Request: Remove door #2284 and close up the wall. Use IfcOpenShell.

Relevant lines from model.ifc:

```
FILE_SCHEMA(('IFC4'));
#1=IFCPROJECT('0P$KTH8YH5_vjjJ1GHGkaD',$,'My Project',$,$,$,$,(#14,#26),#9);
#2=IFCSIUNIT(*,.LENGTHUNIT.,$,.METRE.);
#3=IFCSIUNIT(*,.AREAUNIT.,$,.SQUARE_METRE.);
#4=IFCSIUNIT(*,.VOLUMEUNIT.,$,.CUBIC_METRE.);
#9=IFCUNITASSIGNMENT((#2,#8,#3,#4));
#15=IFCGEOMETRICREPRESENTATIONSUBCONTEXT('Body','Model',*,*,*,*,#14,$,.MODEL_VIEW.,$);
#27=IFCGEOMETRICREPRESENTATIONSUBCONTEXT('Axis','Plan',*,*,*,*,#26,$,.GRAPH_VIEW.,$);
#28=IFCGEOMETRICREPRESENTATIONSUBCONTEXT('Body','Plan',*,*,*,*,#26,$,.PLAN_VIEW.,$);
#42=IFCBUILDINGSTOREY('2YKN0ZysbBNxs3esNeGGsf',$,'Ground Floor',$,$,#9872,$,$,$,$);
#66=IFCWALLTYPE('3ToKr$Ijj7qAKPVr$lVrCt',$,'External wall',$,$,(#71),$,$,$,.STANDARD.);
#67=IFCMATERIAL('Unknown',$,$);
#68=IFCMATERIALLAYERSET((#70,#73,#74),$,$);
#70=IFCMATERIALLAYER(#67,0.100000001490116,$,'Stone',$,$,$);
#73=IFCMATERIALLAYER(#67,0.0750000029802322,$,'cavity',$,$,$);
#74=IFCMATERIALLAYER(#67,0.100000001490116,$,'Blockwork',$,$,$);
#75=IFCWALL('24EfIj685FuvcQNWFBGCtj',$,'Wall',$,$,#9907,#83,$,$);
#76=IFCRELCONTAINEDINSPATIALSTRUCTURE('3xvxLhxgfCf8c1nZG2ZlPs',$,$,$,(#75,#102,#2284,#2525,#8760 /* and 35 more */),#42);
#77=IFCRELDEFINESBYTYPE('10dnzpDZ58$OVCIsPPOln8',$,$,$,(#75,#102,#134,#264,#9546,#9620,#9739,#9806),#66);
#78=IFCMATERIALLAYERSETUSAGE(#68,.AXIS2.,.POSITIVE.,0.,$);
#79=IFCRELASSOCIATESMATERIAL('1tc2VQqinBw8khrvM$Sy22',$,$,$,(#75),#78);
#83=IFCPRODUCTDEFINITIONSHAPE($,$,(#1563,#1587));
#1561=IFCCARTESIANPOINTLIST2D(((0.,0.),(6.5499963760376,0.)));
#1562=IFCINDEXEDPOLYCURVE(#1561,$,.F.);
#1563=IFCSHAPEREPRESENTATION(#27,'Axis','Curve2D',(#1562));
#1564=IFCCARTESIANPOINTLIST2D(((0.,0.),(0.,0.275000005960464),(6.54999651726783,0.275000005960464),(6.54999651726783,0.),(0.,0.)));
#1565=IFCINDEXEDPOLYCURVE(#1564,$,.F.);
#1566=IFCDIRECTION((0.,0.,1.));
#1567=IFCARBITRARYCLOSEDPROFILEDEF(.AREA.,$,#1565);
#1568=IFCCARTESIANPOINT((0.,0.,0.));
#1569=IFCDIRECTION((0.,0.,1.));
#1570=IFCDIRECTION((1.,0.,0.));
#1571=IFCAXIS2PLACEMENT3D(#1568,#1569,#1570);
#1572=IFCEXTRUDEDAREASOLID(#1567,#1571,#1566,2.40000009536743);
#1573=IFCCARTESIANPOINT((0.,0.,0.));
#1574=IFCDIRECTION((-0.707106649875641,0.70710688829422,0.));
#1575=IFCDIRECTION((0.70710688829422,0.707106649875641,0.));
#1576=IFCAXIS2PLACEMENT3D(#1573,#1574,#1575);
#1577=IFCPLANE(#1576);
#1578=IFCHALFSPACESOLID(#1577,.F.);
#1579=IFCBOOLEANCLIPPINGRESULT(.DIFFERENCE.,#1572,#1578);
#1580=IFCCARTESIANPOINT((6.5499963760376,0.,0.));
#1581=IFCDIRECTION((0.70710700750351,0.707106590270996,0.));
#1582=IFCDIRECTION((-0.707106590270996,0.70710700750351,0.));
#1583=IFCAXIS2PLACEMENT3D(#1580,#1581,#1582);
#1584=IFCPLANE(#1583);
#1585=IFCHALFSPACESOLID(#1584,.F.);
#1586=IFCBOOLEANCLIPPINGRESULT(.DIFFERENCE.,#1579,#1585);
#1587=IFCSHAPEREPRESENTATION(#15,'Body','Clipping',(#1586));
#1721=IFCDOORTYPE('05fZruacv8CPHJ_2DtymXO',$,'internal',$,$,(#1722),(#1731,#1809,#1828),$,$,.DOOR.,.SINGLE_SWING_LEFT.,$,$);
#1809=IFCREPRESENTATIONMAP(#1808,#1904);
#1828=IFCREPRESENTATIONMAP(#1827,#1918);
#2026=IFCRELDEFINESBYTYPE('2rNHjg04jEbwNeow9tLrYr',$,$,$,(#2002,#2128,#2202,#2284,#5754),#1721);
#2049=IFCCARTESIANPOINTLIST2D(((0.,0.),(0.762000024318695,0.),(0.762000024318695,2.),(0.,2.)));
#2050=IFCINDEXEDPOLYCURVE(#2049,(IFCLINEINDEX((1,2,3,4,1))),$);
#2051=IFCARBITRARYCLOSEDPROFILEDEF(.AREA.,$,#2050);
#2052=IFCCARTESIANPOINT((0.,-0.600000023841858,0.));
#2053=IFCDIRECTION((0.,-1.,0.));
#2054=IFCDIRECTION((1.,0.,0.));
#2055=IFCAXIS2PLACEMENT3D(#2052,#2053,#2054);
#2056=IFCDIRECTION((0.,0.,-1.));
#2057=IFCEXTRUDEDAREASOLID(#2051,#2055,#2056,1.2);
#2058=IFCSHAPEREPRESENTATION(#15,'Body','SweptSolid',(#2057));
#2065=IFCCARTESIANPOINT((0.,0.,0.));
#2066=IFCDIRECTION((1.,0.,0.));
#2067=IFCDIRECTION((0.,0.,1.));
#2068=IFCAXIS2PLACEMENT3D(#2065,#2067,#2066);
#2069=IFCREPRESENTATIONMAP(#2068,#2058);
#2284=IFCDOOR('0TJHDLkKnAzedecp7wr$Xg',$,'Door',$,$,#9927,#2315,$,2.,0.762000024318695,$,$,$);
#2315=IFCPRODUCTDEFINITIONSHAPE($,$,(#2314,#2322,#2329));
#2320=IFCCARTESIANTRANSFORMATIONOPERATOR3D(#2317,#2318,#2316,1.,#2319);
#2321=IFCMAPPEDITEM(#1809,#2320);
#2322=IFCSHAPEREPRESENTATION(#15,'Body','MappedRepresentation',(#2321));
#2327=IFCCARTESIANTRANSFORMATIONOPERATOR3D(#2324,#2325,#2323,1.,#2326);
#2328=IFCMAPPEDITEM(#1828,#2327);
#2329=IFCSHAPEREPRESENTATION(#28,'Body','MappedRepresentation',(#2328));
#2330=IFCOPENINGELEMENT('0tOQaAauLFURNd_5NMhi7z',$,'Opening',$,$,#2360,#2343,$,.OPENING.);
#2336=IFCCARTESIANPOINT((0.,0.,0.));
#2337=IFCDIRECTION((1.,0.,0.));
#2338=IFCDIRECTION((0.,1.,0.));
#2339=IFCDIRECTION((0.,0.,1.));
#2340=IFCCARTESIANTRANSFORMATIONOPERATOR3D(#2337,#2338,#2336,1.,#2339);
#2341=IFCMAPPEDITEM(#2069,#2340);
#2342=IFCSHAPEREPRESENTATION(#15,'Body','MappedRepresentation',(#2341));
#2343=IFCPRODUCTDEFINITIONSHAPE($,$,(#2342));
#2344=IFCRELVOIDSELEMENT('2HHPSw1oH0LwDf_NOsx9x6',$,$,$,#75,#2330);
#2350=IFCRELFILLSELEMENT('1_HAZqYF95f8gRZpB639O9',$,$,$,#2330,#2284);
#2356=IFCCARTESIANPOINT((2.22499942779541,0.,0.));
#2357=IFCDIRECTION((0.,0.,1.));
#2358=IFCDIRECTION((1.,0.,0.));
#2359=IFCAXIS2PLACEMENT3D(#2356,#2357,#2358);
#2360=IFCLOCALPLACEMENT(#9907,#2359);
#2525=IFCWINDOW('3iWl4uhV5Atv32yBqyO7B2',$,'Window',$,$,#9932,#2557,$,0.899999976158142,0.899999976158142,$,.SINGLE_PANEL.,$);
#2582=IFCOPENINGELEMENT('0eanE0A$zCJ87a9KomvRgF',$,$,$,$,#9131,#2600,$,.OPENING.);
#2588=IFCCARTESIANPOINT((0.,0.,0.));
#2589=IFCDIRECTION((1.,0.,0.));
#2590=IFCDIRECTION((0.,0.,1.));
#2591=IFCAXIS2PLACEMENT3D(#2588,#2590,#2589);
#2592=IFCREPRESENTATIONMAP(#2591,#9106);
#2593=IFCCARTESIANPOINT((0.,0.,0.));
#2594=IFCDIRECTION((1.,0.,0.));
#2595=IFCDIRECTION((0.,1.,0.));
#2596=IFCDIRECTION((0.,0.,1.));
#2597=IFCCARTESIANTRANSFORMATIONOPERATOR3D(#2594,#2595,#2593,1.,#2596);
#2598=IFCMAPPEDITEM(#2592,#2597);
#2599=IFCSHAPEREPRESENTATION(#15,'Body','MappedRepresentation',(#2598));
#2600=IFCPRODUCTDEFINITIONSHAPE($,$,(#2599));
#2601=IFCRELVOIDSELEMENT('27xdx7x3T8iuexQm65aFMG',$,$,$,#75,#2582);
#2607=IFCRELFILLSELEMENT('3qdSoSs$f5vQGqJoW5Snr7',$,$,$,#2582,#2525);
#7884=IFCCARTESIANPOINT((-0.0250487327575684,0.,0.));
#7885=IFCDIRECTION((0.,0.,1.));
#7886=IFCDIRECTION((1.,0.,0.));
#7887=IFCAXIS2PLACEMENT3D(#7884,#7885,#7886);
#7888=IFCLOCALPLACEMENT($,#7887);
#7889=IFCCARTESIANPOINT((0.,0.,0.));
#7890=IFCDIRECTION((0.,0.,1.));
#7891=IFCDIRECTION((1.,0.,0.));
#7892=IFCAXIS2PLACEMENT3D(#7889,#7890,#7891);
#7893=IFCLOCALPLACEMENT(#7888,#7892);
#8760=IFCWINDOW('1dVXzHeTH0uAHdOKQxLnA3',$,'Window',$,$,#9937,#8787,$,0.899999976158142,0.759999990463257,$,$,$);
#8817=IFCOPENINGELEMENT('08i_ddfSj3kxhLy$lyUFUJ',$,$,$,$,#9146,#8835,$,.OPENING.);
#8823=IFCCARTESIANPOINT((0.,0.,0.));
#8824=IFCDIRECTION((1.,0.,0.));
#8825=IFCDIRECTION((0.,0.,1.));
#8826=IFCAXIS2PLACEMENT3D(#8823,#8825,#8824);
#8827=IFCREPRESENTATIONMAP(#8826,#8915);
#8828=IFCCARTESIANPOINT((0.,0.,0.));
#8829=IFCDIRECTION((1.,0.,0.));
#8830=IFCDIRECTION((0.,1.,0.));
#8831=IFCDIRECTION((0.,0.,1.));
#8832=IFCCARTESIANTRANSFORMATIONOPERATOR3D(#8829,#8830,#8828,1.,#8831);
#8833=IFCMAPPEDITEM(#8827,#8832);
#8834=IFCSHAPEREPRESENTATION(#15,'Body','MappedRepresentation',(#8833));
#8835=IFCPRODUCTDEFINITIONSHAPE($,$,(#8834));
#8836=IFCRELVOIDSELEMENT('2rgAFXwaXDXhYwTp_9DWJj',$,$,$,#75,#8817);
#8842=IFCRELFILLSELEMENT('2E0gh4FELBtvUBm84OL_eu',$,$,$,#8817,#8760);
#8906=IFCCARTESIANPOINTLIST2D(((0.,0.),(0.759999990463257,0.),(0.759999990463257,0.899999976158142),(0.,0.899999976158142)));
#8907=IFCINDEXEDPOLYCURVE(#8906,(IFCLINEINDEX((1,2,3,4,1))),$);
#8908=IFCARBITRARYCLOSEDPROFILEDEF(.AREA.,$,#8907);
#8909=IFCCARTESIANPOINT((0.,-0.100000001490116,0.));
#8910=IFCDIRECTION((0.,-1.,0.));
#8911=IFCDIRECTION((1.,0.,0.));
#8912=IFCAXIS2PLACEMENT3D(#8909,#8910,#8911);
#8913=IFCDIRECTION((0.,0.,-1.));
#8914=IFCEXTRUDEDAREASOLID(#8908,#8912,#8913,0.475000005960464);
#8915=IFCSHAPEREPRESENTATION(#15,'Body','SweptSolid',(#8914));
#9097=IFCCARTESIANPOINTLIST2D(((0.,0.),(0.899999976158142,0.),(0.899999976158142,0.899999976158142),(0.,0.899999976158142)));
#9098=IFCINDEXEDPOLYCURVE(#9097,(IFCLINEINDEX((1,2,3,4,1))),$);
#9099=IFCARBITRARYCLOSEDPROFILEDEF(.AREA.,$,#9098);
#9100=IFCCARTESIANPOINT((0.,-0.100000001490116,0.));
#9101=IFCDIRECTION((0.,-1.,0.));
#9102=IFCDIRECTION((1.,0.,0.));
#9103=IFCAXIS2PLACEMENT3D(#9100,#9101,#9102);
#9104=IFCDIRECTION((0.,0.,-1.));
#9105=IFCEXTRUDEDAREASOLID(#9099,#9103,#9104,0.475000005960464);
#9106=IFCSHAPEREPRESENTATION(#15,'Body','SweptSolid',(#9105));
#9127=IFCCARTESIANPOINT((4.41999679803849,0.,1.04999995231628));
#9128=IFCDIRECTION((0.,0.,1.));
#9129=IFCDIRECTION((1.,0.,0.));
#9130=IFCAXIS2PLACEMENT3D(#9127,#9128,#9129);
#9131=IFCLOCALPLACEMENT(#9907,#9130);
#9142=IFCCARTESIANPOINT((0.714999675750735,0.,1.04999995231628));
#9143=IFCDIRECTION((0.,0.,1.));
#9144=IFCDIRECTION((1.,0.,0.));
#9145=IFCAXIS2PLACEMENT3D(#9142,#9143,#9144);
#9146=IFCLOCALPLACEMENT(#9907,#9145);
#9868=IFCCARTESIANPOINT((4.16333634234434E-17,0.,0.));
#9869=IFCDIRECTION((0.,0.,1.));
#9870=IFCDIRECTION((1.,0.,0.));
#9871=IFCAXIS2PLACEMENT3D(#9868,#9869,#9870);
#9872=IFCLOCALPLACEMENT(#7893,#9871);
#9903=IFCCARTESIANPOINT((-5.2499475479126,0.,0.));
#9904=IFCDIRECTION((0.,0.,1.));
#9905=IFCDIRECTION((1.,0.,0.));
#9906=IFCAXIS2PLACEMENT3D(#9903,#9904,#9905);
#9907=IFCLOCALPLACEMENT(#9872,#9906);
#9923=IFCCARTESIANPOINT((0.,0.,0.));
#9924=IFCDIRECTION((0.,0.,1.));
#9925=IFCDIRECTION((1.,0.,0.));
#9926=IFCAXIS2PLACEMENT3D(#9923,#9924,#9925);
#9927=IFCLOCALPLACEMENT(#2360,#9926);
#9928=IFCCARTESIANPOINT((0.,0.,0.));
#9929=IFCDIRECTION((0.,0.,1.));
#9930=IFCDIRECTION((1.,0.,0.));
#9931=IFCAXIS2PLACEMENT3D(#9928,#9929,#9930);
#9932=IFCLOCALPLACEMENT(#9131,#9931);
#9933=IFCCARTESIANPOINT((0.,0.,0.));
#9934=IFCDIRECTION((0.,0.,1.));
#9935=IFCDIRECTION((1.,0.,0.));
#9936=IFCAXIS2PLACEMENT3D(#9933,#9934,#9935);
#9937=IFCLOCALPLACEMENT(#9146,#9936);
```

```python
import ifcopenshell
import ifcopenshell.api.feature
import ifcopenshell.api.root
import ifcopenshell.geom
import ifcopenshell.util.shape

model = ifcopenshell.open("model.ifc")
settings = ifcopenshell.geom.settings()


def volume(element):
    """Net volume in cubic metres, openings subtracted."""
    shape = ifcopenshell.geom.create_shape(settings, element)
    return ifcopenshell.util.shape.get_volume(shape.geometry)


door = model.by_guid("0TJHDLkKnAzedecp7wr$Xg")
opening = door.FillsVoids[0].RelatingOpeningElement
wall = opening.VoidsElements[0].RelatingBuildingElement
before = volume(wall)

ifcopenshell.api.root.remove_product(model, product=door)
ifcopenshell.api.feature.remove_feature(model, feature=opening)

after = volume(wall)

print(f"wall volume {before:.3f} -> {after:.3f} m3")

model.write("model_edited.ifc")
```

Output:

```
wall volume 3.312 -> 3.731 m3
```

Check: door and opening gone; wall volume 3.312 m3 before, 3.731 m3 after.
